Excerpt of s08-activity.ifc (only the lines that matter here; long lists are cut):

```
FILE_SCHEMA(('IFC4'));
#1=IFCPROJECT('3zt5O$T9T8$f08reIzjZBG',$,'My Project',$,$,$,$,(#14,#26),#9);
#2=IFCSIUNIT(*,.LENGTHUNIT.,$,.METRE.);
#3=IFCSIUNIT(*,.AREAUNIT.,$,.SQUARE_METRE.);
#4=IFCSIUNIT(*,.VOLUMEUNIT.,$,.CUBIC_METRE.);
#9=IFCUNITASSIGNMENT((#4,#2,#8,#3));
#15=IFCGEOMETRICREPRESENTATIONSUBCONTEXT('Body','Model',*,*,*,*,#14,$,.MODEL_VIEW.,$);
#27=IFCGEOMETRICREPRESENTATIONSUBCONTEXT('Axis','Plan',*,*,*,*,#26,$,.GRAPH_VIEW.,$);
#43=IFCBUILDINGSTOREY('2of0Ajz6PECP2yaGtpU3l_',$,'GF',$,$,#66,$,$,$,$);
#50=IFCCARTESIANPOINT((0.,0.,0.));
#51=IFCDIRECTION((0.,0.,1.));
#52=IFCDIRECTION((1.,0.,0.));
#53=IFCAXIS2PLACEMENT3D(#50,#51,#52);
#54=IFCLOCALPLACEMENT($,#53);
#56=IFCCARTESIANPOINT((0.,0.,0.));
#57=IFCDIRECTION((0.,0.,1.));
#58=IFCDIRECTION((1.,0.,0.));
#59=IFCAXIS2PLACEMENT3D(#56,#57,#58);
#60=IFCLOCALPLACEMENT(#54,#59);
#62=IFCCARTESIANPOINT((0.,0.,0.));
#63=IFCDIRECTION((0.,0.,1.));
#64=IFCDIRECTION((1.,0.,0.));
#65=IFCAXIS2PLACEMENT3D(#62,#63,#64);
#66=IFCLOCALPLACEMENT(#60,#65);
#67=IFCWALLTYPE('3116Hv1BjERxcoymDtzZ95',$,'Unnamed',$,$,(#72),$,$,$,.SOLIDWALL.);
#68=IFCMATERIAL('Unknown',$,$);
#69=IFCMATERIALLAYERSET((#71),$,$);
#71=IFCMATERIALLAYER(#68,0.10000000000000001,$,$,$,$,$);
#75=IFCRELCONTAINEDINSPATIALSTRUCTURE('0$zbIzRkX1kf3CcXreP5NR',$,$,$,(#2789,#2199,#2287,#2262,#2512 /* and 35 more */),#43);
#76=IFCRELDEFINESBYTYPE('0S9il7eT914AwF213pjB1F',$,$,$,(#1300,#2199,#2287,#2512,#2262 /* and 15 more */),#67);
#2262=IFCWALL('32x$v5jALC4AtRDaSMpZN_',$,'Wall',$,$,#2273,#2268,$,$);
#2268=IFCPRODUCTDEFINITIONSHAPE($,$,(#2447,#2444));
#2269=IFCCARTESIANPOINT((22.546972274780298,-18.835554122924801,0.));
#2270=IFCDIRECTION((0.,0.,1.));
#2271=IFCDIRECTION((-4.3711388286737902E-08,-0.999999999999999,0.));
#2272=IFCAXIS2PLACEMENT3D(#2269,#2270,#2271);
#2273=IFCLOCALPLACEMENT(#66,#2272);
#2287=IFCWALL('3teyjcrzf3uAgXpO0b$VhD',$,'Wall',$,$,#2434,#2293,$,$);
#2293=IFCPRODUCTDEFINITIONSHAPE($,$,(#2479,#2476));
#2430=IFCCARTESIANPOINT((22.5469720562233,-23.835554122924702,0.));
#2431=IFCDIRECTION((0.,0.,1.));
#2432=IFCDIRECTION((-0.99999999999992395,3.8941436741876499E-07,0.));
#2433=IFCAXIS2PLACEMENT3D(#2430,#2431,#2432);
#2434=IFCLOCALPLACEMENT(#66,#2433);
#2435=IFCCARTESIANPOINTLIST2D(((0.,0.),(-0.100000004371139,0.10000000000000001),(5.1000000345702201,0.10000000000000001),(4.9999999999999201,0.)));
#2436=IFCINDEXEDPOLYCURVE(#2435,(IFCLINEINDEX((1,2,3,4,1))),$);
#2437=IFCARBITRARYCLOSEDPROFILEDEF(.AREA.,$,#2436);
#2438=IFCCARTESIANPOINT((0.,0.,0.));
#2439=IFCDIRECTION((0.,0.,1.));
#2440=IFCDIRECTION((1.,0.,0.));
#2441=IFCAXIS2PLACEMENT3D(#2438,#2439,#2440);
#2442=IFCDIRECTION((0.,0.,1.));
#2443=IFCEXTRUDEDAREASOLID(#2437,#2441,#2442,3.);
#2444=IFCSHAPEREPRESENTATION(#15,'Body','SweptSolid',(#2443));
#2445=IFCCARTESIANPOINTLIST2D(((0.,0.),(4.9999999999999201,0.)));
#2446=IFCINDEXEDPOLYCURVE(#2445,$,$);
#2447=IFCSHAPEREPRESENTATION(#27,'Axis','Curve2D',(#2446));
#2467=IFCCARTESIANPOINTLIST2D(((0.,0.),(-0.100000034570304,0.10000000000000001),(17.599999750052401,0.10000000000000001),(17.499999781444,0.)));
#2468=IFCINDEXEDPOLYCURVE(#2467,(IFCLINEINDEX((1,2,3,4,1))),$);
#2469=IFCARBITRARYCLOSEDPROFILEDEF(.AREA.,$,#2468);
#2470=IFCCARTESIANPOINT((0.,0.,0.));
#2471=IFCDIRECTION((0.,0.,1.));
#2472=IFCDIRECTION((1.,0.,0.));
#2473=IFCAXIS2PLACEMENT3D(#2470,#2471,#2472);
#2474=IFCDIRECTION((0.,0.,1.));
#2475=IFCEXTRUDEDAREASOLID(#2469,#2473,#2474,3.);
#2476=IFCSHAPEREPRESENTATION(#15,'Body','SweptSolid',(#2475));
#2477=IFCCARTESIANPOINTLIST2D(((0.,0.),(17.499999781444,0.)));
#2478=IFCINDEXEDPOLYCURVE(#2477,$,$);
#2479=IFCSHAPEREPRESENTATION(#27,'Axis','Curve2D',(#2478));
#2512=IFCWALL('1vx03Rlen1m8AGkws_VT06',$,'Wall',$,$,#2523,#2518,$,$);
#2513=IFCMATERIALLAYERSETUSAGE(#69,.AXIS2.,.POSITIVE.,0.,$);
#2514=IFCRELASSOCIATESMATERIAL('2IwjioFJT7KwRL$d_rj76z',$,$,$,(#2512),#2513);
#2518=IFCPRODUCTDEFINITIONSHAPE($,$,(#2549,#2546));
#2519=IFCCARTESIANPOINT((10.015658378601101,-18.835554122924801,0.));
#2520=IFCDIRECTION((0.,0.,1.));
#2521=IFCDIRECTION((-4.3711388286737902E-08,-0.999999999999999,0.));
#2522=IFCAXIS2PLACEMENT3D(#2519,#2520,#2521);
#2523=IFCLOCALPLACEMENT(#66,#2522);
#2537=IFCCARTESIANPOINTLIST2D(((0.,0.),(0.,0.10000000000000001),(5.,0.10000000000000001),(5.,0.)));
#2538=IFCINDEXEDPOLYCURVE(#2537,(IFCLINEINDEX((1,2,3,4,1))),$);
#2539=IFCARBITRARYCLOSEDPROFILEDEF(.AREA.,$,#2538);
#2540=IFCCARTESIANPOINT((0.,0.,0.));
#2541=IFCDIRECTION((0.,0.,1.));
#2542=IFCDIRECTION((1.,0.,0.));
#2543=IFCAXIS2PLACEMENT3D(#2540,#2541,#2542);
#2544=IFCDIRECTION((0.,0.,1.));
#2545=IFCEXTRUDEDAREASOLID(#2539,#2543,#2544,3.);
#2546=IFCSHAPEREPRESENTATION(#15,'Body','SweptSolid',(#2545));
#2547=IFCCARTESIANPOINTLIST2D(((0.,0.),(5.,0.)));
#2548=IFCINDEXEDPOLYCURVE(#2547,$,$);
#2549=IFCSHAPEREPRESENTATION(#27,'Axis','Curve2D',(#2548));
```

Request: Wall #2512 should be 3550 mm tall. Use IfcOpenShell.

```python
import ifcopenshell
import ifcopenshell.geom
import ifcopenshell.util.representation
import ifcopenshell.util.shape
import ifcopenshell.util.unit

model = ifcopenshell.open("s08-activity.ifc")
unit_scale = ifcopenshell.util.unit.calculate_unit_scale(model)
settings = ifcopenshell.geom.settings()


def volume(element):
    """Net volume in cubic metres, openings subtracted."""
    shape = ifcopenshell.geom.create_shape(settings, element)
    return ifcopenshell.util.shape.get_volume(shape.geometry)


wall = model.by_guid("1vx03Rlen1m8AGkws_VT06")
before = volume(wall)

body = ifcopenshell.util.representation.get_representation(wall, "Model", "Body")
solid = body.Items[0]
old_height = solid.Depth
solid.Depth = 3.55 / unit_scale
after = volume(wall)

print(f"height {old_height:g} -> {solid.Depth:g}, volume {before:.3f} -> {after:.3f} m3")

model.write("s08-activity_v2.ifc")
```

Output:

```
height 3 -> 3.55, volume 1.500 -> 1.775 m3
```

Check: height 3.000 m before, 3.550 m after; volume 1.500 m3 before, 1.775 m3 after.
